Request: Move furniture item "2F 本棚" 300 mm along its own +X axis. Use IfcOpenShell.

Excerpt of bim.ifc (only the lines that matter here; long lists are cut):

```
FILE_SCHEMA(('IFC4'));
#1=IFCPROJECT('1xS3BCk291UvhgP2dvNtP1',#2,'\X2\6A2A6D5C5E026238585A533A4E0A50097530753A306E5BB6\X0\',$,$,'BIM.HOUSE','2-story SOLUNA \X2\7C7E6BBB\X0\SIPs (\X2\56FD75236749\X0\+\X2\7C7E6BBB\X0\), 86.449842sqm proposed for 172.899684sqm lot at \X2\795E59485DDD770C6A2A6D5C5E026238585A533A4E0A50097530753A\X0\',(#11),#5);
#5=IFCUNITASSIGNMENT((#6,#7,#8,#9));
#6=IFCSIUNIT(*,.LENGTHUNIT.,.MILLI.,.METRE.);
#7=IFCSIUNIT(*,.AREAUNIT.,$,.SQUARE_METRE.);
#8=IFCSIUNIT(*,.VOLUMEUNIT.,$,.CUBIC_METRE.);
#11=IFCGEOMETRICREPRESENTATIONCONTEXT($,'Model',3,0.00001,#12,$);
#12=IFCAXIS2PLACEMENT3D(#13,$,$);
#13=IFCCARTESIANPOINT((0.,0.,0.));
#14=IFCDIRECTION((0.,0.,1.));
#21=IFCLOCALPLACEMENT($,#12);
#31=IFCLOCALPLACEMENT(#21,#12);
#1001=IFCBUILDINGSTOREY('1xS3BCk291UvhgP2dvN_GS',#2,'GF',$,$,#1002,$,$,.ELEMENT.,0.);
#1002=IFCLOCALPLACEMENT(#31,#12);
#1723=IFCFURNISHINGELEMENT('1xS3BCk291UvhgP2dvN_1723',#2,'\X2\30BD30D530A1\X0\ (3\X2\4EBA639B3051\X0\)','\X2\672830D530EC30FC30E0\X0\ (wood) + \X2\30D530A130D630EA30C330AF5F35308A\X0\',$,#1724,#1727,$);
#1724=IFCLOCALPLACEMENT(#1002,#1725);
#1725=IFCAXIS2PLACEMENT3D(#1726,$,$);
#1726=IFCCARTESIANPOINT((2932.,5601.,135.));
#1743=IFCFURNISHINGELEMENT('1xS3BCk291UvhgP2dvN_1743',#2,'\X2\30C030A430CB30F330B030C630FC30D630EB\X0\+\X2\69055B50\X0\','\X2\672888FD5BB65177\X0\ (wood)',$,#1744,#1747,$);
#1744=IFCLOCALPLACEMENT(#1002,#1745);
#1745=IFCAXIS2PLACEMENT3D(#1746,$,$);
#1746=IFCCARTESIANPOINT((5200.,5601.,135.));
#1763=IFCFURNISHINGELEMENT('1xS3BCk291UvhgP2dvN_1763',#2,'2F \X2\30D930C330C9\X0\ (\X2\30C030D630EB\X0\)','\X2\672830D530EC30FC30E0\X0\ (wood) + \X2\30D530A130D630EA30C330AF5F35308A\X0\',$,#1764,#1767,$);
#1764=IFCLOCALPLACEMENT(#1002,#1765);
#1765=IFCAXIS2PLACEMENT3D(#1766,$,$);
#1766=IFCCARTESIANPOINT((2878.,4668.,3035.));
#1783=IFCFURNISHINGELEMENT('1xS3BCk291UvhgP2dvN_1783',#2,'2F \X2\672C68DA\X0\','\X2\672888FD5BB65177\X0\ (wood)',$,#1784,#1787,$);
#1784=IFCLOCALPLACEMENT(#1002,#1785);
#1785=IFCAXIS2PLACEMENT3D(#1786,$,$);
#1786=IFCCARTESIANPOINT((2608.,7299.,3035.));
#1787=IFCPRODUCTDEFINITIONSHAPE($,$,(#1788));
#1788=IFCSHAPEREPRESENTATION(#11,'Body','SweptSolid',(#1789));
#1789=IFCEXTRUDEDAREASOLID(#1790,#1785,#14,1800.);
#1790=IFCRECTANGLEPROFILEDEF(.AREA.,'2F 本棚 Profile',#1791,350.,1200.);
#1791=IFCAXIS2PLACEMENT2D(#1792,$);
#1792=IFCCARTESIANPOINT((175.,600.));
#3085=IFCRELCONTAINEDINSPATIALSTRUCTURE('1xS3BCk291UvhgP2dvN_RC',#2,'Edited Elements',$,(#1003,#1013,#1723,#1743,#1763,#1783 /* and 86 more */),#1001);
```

```python
import ifcopenshell
import ifcopenshell.api.geometry
import ifcopenshell.util.placement

model = ifcopenshell.open("bim.ifc")

item = model.by_guid("1xS3BCk291UvhgP2dvN_1783")
matrix = ifcopenshell.util.placement.get_local_placement(item.ObjectPlacement)
matrix[:3, 3] += matrix[:3, 0] * 300.0
ifcopenshell.api.geometry.edit_object_placement(model, product=item, matrix=matrix, is_si=False)

print(ifcopenshell.util.placement.get_local_placement(item.ObjectPlacement).round(3) + 0.0)

model.write("bim_v2.ifc")
```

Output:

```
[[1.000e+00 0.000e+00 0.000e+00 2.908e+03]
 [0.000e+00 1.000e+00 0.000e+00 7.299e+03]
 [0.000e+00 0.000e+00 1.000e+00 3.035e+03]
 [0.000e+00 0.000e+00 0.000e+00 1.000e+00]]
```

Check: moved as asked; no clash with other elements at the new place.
